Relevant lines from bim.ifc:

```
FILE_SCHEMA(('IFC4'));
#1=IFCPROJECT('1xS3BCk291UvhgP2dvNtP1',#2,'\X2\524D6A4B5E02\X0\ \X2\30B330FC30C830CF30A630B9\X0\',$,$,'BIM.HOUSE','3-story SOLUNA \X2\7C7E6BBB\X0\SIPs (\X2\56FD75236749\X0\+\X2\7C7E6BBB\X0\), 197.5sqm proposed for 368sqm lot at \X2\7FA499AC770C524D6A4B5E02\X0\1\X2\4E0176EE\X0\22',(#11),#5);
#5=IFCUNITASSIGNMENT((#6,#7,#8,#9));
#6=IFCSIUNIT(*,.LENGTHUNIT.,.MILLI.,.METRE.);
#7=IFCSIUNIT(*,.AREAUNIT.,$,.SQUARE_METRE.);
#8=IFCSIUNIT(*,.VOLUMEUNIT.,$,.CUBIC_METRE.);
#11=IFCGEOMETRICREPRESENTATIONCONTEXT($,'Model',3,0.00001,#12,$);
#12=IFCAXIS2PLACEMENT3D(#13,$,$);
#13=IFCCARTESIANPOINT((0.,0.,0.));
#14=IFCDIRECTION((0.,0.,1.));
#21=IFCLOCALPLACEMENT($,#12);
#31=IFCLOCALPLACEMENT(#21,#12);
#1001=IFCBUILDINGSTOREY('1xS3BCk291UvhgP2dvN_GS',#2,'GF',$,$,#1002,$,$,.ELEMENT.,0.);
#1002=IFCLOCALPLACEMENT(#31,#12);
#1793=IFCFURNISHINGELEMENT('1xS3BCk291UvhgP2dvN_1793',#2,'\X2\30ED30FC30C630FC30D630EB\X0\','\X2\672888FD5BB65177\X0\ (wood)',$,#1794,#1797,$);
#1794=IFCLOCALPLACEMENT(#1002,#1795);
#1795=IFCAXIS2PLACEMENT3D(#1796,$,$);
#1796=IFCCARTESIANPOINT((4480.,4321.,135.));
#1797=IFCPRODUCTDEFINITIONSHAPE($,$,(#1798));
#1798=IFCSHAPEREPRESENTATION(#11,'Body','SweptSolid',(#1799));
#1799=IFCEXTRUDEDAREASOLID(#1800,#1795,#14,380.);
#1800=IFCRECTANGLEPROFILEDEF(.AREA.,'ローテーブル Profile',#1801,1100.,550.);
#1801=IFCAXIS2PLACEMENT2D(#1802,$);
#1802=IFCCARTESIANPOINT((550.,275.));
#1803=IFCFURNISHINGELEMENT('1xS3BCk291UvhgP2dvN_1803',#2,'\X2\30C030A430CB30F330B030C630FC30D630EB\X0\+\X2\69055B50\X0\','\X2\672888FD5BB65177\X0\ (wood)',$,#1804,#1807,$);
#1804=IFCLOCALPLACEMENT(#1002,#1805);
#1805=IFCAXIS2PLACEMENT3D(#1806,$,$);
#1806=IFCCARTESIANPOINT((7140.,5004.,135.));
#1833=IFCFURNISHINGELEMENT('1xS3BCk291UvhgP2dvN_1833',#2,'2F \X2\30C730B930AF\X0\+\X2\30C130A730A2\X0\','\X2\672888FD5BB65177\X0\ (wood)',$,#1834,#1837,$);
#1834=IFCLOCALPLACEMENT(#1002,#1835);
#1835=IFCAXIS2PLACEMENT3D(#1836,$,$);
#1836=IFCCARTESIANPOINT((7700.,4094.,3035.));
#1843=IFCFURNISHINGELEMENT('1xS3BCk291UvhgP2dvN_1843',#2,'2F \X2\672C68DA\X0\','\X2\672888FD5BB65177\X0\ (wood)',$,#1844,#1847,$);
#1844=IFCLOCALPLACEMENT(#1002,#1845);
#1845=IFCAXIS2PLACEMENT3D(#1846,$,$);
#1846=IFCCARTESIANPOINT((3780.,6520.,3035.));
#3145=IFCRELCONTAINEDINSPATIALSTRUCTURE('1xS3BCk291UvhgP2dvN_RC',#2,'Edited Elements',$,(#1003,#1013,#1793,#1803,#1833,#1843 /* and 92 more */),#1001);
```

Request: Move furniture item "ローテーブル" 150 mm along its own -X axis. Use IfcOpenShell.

```python
import ifcopenshell
import ifcopenshell.api.geometry
import ifcopenshell.util.placement
import ifcopenshell.util.unit

model = ifcopenshell.open("bim.ifc")
unit_scale = ifcopenshell.util.unit.calculate_unit_scale(model)

item = model.by_guid("1xS3BCk291UvhgP2dvN_1793")
matrix = ifcopenshell.util.placement.get_local_placement(item.ObjectPlacement)
matrix[:3, 3] -= matrix[:3, 0] * 0.15 / unit_scale
ifcopenshell.api.geometry.edit_object_placement(model, product=item, matrix=matrix, is_si=False)

print(ifcopenshell.util.placement.get_local_placement(item.ObjectPlacement).round(3) + 0.0)

model.write("bim_rev.ifc")
```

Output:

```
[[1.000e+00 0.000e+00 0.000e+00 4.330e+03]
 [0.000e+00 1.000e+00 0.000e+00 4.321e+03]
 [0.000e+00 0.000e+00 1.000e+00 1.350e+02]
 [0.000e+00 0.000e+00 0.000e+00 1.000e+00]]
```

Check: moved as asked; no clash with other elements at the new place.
